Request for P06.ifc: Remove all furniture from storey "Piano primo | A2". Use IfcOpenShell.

First a look at what the model holds.

```python
import ifcopenshell
import ifcopenshell.util.element

model = ifcopenshell.open("P06.ifc")
print(model.schema)
storey = next(s for s in model.by_type("IfcBuildingStorey") if s.Name == "Piano primo | A2")
furniture = [e for e in ifcopenshell.util.element.get_decomposition(storey) if e.is_a("IfcFurnishingElement")]
seen = {}
for e in furniture:
    element_type = ifcopenshell.util.element.get_type(e)
    name = element_type.Name if element_type not in (None, e) else None
    seen[name] = seen.get(name, 0) + 1
for name, count in sorted(seen.items(), key=str):
    print(count, "x", name)
```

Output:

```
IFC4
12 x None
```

```python
import ifcopenshell
import ifcopenshell.api.root
import ifcopenshell.util.element

model = ifcopenshell.open("P06.ifc")

storey = next(s for s in model.by_type("IfcBuildingStorey") if s.Name == "Piano primo | A2")
furniture = [e for e in ifcopenshell.util.element.get_decomposition(storey) if e.is_a("IfcFurnishingElement")]

for e in furniture:
    ifcopenshell.api.root.remove_product(model, product=e)
print(len(furniture), "removed")

model.write("P06_updated.ifc")
```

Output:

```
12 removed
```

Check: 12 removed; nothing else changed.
